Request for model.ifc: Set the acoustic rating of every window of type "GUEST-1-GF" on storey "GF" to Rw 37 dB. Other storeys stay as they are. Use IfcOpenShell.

First a look at what the model holds.

```python
import ifcopenshell
import ifcopenshell.util.element

model = ifcopenshell.open("model.ifc")
print(model.schema)
storey = next(s for s in model.by_type("IfcBuildingStorey") if s.Name == "GF")
windows = [e for e in ifcopenshell.util.element.get_decomposition(storey) if e.is_a("IfcWindow")]
seen = {}
for e in windows:
    element_type = ifcopenshell.util.element.get_type(e)
    key = (element_type.Name if element_type != e and element_type else None, ifcopenshell.util.element.get_pset(e, "Pset_WindowCommon", "AcousticRating"))
    seen[key] = seen.get(key, 0) + 1
for (name, value), count in sorted(seen.items(), key=str):
    print(count, "x", name, "|", value)
```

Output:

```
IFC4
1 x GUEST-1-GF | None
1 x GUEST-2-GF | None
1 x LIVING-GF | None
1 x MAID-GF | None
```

```python
import ifcopenshell
import ifcopenshell.api.pset
import ifcopenshell.util.element

model = ifcopenshell.open("model.ifc")

storey = next(s for s in model.by_type("IfcBuildingStorey") if s.Name == "GF")
windows = [e for e in ifcopenshell.util.element.get_decomposition(storey) if e.is_a("IfcWindow")]

count = 0
for e in windows:
    element_type = ifcopenshell.util.element.get_type(e)
    if element_type in (None, e) or element_type.Name != "GUEST-1-GF":
        continue
    # add_pset returns the element's existing set when there is one.
    pset = ifcopenshell.api.pset.add_pset(model, product=e, name="Pset_WindowCommon")
    ifcopenshell.api.pset.edit_pset(model, pset=pset, properties={"AcousticRating": "Rw 37 dB"})
    count += 1

print(count, "windows updated")

model.write("model_updated.ifc")
```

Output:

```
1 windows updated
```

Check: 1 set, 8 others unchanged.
